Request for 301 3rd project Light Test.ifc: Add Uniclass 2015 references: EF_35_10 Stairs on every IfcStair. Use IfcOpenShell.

First a look at what the model holds.

```python
import ifcopenshell

model = ifcopenshell.open("301 3rd project Light Test.ifc")
print(model.schema)
print("classifications:", [c.Name for c in model.by_type("IfcClassification")])
for ifc_class in ("IfcDoor", "IfcRoof", "IfcStair", "IfcWall", "IfcWindow"):
    print(ifc_class, len(model.by_type(ifc_class)))
```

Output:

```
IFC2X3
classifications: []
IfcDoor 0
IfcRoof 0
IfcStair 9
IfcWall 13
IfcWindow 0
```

```python
import ifcopenshell
import ifcopenshell.api.classification

model = ifcopenshell.open("301 3rd project Light Test.ifc")

# IFC2X3 requires Source and Edition and has no link from the project to the system.
system = model.create_entity("IfcClassification", Source="NBS", Edition="2015", Name="Uniclass 2015")

codes = {
    "IfcStair": ("EF_35_10", "Stairs"),
}
for ifc_class, (code, name) in codes.items():
    products = model.by_type(ifc_class)
    ifcopenshell.api.classification.add_reference(
        model, products=products, classification=system, identification=code, name=name
    )
    print(code, len(products))

model.write("301 3rd project Light Test_edited.ifc")
```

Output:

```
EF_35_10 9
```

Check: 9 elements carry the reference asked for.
